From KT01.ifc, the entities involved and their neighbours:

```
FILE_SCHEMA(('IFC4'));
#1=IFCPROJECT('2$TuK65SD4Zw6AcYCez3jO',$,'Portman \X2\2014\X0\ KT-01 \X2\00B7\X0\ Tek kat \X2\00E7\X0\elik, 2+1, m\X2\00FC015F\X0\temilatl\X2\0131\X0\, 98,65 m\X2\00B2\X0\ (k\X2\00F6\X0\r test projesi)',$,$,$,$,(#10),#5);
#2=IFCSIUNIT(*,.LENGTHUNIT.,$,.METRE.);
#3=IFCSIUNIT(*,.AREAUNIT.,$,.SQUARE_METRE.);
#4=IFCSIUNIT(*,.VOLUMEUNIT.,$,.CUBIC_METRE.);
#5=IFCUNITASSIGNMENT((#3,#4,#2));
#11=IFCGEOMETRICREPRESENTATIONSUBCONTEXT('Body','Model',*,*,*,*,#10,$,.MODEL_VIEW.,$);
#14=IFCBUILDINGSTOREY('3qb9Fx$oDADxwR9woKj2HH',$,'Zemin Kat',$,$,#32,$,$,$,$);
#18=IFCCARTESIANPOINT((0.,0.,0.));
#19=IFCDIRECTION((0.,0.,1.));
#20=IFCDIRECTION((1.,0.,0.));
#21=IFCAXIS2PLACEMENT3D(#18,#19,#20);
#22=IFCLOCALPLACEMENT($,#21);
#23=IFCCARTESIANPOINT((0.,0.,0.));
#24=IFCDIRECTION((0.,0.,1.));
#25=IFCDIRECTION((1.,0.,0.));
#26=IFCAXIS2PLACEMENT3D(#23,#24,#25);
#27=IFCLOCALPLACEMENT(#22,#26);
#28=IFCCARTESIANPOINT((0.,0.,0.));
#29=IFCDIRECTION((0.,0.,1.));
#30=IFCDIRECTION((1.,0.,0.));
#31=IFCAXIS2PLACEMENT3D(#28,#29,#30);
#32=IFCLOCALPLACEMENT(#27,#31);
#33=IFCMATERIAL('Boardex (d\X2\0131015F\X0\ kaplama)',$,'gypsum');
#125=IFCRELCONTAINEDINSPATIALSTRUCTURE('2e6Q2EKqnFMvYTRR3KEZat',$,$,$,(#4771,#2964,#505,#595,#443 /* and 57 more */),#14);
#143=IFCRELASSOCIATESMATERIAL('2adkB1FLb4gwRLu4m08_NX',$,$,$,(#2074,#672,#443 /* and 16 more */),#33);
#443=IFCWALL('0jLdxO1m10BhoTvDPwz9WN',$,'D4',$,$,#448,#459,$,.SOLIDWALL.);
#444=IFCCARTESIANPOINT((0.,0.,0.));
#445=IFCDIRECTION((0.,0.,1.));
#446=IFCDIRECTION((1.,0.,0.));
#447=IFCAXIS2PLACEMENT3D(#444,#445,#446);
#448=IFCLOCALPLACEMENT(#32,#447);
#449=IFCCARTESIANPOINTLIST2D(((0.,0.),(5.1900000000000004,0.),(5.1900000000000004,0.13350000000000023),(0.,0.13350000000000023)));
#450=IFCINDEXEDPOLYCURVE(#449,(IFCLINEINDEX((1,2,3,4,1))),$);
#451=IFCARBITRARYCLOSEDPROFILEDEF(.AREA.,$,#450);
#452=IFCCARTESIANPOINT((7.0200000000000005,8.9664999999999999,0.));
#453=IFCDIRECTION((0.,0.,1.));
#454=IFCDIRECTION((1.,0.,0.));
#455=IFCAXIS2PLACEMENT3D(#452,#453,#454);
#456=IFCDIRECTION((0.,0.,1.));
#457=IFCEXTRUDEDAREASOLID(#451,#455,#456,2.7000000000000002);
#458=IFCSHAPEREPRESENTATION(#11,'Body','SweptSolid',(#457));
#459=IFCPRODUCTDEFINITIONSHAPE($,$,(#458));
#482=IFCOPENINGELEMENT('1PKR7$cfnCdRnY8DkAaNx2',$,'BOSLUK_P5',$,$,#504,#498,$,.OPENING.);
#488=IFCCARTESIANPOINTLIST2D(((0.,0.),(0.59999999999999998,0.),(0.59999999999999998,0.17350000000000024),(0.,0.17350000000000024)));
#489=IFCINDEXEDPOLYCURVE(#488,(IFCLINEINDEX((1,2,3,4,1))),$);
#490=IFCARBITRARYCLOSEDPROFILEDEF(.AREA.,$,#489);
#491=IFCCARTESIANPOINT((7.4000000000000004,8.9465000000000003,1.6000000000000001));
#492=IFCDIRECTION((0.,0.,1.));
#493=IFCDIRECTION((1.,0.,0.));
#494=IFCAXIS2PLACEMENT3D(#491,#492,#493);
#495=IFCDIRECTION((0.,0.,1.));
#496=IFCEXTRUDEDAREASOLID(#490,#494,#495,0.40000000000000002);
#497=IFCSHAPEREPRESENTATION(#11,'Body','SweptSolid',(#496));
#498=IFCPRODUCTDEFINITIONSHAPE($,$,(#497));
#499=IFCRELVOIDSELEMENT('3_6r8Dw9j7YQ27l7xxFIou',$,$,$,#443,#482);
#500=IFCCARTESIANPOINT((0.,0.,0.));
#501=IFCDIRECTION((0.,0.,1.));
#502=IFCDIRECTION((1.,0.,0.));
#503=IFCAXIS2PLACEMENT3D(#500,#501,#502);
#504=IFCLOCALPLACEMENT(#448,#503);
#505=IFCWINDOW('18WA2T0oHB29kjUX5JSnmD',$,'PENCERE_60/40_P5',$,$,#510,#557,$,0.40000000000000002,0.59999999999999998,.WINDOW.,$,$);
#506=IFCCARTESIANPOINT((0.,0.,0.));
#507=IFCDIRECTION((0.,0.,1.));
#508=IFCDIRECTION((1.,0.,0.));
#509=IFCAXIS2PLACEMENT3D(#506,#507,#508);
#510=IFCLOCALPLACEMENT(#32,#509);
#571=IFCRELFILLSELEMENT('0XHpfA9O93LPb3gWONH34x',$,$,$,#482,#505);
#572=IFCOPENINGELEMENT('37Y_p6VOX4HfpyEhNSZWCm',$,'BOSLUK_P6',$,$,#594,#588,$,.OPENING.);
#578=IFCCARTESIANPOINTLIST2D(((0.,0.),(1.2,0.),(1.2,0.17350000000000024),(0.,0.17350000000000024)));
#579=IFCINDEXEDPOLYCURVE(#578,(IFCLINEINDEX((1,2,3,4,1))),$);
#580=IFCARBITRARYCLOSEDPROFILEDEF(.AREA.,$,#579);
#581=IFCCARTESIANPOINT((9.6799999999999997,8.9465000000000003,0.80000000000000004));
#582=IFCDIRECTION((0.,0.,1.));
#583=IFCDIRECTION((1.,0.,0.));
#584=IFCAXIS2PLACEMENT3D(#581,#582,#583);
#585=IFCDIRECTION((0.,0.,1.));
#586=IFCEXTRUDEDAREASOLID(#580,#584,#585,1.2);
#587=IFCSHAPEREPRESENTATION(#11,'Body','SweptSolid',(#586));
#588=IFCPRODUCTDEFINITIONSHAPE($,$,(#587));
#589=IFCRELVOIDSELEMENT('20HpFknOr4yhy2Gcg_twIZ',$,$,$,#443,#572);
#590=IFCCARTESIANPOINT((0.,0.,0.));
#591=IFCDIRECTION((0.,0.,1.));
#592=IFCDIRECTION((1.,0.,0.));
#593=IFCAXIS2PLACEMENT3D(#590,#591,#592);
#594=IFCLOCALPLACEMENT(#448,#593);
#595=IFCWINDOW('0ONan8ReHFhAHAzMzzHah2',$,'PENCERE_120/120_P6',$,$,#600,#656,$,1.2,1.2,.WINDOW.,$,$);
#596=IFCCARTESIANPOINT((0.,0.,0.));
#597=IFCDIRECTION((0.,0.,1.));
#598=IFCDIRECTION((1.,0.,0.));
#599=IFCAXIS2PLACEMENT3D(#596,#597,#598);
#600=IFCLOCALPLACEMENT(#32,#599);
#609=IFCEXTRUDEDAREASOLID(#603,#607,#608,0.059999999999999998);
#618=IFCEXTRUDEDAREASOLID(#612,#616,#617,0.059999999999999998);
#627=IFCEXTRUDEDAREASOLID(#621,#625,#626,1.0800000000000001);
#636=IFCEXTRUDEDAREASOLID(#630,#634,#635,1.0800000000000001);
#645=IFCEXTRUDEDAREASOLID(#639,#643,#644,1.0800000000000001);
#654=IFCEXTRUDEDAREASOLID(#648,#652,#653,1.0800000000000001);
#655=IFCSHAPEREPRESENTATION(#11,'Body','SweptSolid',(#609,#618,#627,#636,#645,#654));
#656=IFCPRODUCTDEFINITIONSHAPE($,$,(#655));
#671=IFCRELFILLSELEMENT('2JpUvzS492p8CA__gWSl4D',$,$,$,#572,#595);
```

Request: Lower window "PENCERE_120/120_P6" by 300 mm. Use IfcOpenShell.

```python
import numpy as np
import ifcopenshell
import ifcopenshell.api.geometry
import ifcopenshell.util.placement
import ifcopenshell.util.unit

model = ifcopenshell.open("KT01.ifc")
unit_scale = ifcopenshell.util.unit.calculate_unit_scale(model)

window = model.by_guid("0ONan8ReHFhAHAzMzzHah2")
opening = window.FillsVoids[0].RelatingOpeningElement
dz = -0.3 / unit_scale

shift = np.array([0.0, 0.0, dz])
# The window is not placed relative to its opening, so move both.
for product in (opening, window):
    matrix = ifcopenshell.util.placement.get_local_placement(product.ObjectPlacement)
    matrix[:3, 3] += shift
    ifcopenshell.api.geometry.edit_object_placement(model, product=product, matrix=matrix, is_si=False)

print(f"moved by {dz * unit_scale:+.3f} m")

model.write("KT01_rev.ifc")
```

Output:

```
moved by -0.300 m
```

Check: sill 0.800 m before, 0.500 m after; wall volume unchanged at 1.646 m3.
